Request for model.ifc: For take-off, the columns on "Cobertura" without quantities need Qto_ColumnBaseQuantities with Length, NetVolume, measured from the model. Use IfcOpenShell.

First a look at what the model holds.

```python
import ifcopenshell
import ifcopenshell.util.element
import ifcopenshell.util.unit

model = ifcopenshell.open("model.ifc")
print(model.schema)
for unit_type in ("LENGTHUNIT", "AREAUNIT", "VOLUMEUNIT"):
    print(unit_type, ifcopenshell.util.unit.calculate_unit_scale(model, unit_type))
storey = next(s for s in model.by_type("IfcBuildingStorey") if s.Name == "Cobertura")
columns = [e for e in ifcopenshell.util.element.get_decomposition(storey) if e.is_a("IfcColumn")]
for e in sorted(columns, key=lambda e: e.id()):
    print(e.id(), e.is_a(), e.Name, list(ifcopenshell.util.element.get_psets(e, qtos_only=True)), sep=" | ")
```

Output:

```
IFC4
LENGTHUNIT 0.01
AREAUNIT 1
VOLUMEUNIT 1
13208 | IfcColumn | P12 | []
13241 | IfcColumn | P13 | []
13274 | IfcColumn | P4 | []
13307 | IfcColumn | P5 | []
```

```python
import ifcopenshell
import ifcopenshell.api.pset
import ifcopenshell.geom
import ifcopenshell.util.element
import ifcopenshell.util.shape
import ifcopenshell.util.unit

model = ifcopenshell.open("model.ifc")
unit_scale = ifcopenshell.util.unit.calculate_unit_scale(model)
volume_scale = ifcopenshell.util.unit.calculate_unit_scale(model, "VOLUMEUNIT")
settings = ifcopenshell.geom.settings()

storey = next(s for s in model.by_type("IfcBuildingStorey") if s.Name == "Cobertura")
columns = [e for e in ifcopenshell.util.element.get_decomposition(storey) if e.is_a("IfcColumn")]

for e in sorted(columns, key=lambda e: e.id()):
    if ifcopenshell.util.element.get_psets(e, qtos_only=True, should_inherit=False):
        continue
    # Geometry comes back in metres, in the element's own axes.
    shape = ifcopenshell.geom.create_shape(settings, e)
    values = {
        "Length": ifcopenshell.util.shape.get_z(shape.geometry) / unit_scale,
        "NetVolume": ifcopenshell.util.shape.get_volume(shape.geometry) / volume_scale,
    }
    qto = ifcopenshell.api.pset.add_qto(model, product=e, name="Qto_ColumnBaseQuantities")
    ifcopenshell.api.pset.edit_qto(model, qto=qto, properties=values)
    print(e.id(), {k: round(v, 3) for k, v in values.items()})

model.write("model_edited.ifc")
```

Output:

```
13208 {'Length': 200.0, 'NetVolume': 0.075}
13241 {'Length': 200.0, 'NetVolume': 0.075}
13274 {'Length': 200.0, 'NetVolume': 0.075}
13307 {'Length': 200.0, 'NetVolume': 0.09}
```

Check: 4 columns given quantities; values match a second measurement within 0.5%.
